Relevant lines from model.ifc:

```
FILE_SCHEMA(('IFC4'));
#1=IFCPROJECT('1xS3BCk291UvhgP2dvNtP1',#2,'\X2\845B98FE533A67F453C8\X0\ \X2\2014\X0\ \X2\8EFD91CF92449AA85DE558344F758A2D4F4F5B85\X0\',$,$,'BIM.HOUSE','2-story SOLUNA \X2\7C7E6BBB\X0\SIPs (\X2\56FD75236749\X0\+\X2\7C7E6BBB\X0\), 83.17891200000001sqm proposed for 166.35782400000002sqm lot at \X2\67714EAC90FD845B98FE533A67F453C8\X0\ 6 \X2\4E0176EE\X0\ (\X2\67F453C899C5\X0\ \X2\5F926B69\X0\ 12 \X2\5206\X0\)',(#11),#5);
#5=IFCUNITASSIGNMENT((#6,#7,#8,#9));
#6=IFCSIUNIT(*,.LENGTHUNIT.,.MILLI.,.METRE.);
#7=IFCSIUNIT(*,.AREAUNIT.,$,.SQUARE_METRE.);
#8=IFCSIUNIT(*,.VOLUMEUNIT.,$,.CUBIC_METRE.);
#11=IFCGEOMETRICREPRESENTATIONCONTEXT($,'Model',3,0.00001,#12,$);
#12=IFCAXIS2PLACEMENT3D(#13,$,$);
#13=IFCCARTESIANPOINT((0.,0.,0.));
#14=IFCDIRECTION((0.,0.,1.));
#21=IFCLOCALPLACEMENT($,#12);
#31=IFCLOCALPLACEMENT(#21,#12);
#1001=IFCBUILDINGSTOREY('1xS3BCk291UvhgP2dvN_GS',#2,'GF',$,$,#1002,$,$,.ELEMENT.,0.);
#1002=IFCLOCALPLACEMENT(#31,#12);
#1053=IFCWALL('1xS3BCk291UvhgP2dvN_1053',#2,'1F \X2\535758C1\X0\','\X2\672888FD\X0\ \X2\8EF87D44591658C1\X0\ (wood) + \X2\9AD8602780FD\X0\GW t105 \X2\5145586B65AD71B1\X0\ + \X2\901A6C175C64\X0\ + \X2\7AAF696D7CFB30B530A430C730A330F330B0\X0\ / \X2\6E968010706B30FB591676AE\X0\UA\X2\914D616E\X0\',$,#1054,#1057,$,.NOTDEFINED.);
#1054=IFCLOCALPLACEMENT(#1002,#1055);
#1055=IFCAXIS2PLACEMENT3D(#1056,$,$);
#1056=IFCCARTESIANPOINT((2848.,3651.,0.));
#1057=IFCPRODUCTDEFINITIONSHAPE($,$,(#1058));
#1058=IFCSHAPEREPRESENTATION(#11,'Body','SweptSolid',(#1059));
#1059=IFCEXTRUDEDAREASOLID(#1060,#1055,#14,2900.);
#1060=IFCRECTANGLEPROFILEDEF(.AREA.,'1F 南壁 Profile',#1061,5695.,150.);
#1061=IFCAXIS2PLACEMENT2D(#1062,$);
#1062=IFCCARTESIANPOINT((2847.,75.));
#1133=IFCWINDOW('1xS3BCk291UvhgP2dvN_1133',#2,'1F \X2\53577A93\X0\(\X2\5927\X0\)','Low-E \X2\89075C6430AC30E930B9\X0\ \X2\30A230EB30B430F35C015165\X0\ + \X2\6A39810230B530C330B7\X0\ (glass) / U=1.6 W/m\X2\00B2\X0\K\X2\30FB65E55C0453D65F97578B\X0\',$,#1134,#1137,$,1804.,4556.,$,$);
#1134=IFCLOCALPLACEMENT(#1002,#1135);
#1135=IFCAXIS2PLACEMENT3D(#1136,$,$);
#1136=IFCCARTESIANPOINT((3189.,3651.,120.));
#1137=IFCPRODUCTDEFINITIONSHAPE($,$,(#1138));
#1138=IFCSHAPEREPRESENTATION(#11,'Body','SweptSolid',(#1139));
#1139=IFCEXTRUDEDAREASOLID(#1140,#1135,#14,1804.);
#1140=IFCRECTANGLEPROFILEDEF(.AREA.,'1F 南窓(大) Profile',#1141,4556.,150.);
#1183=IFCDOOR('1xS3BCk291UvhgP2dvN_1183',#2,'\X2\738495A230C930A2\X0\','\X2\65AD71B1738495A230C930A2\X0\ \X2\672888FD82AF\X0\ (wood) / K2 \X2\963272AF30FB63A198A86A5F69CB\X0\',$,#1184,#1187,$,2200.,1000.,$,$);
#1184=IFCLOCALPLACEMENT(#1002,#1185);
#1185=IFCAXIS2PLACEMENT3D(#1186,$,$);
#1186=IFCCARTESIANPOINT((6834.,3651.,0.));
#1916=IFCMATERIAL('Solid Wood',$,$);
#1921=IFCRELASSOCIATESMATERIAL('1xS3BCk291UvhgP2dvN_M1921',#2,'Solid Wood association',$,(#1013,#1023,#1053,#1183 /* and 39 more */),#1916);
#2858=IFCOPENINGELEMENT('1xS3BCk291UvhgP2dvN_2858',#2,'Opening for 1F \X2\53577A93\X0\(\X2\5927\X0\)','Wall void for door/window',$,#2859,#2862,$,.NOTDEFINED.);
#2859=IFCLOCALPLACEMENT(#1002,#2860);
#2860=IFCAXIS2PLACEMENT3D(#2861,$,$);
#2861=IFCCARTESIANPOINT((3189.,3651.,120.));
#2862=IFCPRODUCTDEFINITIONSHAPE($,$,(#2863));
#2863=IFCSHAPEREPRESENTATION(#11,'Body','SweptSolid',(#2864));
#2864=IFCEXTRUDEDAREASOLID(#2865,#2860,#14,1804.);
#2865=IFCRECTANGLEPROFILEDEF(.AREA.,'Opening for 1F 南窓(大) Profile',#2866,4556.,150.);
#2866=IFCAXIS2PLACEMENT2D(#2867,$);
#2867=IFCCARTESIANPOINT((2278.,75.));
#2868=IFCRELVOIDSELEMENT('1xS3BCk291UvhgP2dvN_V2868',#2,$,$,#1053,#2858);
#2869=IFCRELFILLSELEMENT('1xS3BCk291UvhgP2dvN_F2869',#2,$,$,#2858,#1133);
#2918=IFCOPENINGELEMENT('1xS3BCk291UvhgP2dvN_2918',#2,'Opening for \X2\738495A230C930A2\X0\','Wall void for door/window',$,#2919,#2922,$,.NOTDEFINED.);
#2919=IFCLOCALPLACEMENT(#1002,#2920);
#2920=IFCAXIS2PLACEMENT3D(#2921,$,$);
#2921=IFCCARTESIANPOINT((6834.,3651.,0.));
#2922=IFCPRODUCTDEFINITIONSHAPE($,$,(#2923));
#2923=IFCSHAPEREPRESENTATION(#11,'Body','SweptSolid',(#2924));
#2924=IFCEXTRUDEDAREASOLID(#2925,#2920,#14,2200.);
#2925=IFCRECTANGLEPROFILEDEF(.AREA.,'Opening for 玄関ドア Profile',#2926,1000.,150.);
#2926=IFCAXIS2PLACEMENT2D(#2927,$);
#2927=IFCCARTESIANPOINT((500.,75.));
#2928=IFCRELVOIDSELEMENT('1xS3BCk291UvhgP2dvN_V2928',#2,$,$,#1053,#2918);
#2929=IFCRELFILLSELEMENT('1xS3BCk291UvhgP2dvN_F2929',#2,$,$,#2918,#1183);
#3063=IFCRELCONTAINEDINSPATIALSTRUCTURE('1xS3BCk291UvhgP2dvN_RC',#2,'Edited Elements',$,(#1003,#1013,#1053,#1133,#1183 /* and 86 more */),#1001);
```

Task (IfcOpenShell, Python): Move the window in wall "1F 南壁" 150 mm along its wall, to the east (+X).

```python
import ifcopenshell
import ifcopenshell.api.geometry
import ifcopenshell.util.placement
import ifcopenshell.util.unit

model = ifcopenshell.open("model.ifc")
unit_scale = ifcopenshell.util.unit.calculate_unit_scale(model)

window = model.by_id(1133)
opening = window.FillsVoids[0].RelatingOpeningElement
wall = opening.VoidsElements[0].RelatingBuildingElement

wall_matrix = ifcopenshell.util.placement.get_local_placement(wall.ObjectPlacement)
shift = wall_matrix[:3, 0] * 0.15 / unit_scale
before = ifcopenshell.util.placement.get_local_placement(window.ObjectPlacement)[:3, 3].copy()

# The window is not placed relative to its opening, so move both.
for product in (opening, window):
    matrix = ifcopenshell.util.placement.get_local_placement(product.ObjectPlacement)
    matrix[:3, 3] += shift
    ifcopenshell.api.geometry.edit_object_placement(model, product=product, matrix=matrix, is_si=False)

after = ifcopenshell.util.placement.get_local_placement(window.ObjectPlacement)[:3, 3]
print("window moved by", (after - before).round(3) + 0.0)

model.write("model_updated.ifc")
```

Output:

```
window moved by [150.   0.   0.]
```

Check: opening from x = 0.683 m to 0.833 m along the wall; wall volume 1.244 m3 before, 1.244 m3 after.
